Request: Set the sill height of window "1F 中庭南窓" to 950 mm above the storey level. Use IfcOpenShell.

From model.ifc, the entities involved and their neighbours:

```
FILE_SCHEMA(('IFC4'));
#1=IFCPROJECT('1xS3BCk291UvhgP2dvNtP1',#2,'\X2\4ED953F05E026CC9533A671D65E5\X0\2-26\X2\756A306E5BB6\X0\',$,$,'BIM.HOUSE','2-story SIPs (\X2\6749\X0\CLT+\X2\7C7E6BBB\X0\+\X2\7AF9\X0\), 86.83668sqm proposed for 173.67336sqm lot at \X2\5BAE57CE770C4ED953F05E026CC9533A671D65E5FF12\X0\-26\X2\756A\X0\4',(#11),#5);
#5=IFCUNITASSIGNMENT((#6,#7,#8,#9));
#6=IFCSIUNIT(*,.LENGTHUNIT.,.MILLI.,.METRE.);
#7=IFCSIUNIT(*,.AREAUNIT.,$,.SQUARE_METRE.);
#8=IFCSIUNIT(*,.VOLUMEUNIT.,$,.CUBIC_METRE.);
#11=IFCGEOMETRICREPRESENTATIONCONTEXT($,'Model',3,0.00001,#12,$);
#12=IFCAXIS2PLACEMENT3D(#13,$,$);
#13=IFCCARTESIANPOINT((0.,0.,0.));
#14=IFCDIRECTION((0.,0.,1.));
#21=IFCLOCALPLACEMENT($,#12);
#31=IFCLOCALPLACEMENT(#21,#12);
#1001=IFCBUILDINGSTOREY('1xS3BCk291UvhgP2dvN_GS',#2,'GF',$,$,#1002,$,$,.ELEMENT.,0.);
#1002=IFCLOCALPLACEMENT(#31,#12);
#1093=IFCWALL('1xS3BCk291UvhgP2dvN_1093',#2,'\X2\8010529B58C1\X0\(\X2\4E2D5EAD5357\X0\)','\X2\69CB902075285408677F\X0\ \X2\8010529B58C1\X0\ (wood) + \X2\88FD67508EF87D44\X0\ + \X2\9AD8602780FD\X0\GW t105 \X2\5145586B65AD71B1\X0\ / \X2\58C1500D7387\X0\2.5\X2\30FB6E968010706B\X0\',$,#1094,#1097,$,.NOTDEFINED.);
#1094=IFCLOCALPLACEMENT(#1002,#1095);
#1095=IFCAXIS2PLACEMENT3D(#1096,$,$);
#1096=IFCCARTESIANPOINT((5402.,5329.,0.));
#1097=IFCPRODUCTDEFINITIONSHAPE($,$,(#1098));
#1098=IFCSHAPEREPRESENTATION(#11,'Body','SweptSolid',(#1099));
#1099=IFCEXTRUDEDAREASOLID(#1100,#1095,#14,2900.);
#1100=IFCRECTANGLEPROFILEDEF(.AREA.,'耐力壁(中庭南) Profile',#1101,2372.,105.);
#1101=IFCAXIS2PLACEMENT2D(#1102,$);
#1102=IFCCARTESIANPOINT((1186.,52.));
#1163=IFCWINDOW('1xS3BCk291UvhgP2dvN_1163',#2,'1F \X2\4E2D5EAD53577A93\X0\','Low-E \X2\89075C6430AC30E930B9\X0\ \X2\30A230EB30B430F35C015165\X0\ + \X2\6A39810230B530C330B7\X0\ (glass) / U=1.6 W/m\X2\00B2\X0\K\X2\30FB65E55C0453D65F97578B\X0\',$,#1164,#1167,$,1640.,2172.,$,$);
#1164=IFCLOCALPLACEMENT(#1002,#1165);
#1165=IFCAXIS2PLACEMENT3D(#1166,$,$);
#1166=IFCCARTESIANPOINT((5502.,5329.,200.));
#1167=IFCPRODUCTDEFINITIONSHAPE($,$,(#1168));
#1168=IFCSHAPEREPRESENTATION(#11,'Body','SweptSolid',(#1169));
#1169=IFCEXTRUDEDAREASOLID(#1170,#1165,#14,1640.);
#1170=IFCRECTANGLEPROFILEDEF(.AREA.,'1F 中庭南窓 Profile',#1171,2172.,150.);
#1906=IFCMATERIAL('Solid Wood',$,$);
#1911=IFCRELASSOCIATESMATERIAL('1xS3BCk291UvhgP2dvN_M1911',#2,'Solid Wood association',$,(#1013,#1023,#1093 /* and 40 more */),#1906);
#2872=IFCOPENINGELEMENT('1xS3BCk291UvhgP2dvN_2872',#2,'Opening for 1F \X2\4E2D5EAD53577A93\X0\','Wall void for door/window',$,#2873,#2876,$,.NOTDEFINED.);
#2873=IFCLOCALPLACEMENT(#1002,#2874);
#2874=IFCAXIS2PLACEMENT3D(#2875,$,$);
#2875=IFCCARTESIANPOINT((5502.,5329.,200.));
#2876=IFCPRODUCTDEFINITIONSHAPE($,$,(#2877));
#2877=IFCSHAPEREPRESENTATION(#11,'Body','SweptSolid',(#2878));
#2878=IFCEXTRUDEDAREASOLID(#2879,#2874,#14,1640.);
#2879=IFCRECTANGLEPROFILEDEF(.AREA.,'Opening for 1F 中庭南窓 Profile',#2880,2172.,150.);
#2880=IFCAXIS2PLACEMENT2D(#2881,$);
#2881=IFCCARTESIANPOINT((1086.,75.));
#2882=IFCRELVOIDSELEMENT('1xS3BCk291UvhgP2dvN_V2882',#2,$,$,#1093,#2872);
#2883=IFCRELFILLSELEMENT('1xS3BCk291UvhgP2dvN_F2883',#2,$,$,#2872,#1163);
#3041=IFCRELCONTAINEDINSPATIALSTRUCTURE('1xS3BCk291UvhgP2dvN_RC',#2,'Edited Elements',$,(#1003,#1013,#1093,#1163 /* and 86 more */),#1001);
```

```python
import numpy as np
import ifcopenshell
import ifcopenshell.api.geometry
import ifcopenshell.geom
import ifcopenshell.util.element
import ifcopenshell.util.placement
import ifcopenshell.util.shape
import ifcopenshell.util.unit

model = ifcopenshell.open("model.ifc")
unit_scale = ifcopenshell.util.unit.calculate_unit_scale(model)

window = model.by_id(1163)
opening = window.FillsVoids[0].RelatingOpeningElement
storey = ifcopenshell.util.element.get_container(window, ifc_class="IfcBuildingStorey")
level = ifcopenshell.util.placement.get_local_placement(storey.ObjectPlacement)[2, 3]

# The opening's origin need not be at the sill, so measure its lowest point.
shape = ifcopenshell.geom.create_shape(ifcopenshell.geom.settings(), opening)
bottom = ifcopenshell.util.shape.get_shape_bottom_elevation(shape, shape.geometry) / unit_scale
dz = level + 950.0 - bottom

shift = np.array([0.0, 0.0, dz])
# The window is not placed relative to its opening, so move both.
for product in (opening, window):
    matrix = ifcopenshell.util.placement.get_local_placement(product.ObjectPlacement)
    matrix[:3, 3] += shift
    ifcopenshell.api.geometry.edit_object_placement(model, product=product, matrix=matrix, is_si=False)

print(f"moved by {dz * unit_scale:+.3f} m")

model.write("model_edited.ifc")
```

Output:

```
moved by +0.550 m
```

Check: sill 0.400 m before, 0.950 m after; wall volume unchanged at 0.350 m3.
